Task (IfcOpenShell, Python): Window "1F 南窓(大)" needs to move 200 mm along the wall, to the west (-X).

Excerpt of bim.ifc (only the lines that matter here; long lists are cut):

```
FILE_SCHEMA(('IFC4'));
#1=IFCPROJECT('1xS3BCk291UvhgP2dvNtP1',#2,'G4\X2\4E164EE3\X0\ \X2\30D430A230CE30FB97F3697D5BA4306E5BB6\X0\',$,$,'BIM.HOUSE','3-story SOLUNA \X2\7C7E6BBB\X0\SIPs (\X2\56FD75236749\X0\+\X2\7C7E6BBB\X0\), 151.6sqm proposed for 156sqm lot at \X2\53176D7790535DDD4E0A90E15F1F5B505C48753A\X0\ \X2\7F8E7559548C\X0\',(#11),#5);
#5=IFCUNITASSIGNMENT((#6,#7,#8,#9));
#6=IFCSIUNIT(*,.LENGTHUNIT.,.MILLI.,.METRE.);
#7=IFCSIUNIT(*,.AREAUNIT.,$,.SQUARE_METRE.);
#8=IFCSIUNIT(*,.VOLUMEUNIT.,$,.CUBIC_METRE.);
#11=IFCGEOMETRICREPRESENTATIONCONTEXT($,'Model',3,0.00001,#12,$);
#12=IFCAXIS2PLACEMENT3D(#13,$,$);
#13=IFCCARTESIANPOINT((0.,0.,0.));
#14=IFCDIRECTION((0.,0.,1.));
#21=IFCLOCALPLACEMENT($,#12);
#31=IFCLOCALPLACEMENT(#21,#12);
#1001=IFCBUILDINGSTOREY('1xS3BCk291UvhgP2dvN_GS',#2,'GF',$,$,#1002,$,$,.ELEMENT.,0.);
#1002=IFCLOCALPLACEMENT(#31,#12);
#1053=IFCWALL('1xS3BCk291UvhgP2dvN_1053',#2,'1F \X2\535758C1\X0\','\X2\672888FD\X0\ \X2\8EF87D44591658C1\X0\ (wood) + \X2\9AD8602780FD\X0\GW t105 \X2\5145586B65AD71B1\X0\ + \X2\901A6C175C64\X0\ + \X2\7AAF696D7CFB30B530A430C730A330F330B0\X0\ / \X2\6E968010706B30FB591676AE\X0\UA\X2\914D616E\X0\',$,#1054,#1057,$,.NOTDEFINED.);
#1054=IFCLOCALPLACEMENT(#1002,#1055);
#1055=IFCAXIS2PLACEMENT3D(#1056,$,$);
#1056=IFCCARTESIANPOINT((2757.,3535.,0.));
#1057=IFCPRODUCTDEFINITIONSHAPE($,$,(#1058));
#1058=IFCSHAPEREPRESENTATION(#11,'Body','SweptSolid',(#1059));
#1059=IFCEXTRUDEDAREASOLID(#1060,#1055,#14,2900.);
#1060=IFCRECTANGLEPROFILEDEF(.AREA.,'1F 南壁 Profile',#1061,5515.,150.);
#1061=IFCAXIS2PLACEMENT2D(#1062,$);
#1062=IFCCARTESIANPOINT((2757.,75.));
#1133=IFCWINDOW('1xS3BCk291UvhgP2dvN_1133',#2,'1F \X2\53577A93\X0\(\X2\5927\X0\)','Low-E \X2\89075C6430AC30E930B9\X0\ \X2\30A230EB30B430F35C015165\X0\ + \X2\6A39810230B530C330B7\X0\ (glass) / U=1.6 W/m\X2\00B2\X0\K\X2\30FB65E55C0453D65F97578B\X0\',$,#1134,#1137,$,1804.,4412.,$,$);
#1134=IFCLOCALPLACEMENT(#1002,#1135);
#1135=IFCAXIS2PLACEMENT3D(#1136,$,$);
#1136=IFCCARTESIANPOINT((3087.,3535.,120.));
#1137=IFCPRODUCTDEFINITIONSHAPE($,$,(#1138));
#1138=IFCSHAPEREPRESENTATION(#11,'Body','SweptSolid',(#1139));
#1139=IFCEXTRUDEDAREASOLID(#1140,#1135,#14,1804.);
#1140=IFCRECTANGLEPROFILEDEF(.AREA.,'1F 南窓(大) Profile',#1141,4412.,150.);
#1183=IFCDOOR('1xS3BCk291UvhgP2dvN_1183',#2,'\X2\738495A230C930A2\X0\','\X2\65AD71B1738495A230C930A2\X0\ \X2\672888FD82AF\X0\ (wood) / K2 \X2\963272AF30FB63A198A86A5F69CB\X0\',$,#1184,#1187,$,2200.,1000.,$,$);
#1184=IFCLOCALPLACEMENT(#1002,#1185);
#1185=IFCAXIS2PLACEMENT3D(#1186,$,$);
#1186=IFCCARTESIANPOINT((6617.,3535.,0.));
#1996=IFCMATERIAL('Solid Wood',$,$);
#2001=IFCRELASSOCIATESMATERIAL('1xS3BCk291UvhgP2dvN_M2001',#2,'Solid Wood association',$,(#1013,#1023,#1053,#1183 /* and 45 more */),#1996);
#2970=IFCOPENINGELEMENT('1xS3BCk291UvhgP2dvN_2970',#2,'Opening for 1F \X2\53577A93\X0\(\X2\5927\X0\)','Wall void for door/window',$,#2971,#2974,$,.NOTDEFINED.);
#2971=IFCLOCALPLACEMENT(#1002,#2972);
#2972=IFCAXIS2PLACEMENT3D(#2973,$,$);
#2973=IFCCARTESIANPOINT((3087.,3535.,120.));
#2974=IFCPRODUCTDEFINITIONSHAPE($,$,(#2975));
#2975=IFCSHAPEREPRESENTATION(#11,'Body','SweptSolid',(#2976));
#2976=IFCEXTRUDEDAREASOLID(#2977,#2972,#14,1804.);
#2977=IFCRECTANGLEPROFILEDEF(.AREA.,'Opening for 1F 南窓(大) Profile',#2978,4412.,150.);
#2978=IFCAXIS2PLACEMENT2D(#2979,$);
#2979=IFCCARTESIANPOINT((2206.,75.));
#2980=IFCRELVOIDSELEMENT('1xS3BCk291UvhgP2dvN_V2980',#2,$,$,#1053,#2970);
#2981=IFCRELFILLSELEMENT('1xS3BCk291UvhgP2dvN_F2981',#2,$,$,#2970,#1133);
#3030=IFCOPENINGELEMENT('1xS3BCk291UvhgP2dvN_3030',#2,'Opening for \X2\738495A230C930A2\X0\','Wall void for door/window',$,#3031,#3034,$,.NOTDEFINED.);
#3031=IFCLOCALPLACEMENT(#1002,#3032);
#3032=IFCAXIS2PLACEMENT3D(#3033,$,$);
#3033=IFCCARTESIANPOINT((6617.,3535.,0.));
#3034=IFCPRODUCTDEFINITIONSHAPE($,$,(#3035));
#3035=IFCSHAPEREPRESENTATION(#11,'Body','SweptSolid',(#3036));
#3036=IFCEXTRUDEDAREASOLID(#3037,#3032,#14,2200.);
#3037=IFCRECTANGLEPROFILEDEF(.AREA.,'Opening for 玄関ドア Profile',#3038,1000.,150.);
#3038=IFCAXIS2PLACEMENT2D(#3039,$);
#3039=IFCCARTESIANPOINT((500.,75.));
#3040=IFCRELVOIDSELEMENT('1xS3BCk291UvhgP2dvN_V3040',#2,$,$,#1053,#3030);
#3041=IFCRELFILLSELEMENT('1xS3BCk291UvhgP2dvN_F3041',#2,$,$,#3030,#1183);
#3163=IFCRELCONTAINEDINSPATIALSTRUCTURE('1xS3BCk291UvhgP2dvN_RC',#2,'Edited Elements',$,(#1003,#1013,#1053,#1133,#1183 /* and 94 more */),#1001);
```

```python
import ifcopenshell
import ifcopenshell.api.geometry
import ifcopenshell.util.placement
import ifcopenshell.util.unit

model = ifcopenshell.open("bim.ifc")
unit_scale = ifcopenshell.util.unit.calculate_unit_scale(model)

window = model.by_guid("1xS3BCk291UvhgP2dvN_1133")
opening = window.FillsVoids[0].RelatingOpeningElement
wall = opening.VoidsElements[0].RelatingBuildingElement

wall_matrix = ifcopenshell.util.placement.get_local_placement(wall.ObjectPlacement)
shift = wall_matrix[:3, 0] * -0.2 / unit_scale
before = ifcopenshell.util.placement.get_local_placement(window.ObjectPlacement)[:3, 3].copy()

# The window is not placed relative to its opening, so move both.
for product in (opening, window):
    matrix = ifcopenshell.util.placement.get_local_placement(product.ObjectPlacement)
    matrix[:3, 3] += shift
    ifcopenshell.api.geometry.edit_object_placement(model, product=product, matrix=matrix, is_si=False)

after = ifcopenshell.util.placement.get_local_placement(window.ObjectPlacement)[:3, 3]
print("window moved by", (after - before).round(3) + 0.0)

model.write("bim_edited.ifc")
```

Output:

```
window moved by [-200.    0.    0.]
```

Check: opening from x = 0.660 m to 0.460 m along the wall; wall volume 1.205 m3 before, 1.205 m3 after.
